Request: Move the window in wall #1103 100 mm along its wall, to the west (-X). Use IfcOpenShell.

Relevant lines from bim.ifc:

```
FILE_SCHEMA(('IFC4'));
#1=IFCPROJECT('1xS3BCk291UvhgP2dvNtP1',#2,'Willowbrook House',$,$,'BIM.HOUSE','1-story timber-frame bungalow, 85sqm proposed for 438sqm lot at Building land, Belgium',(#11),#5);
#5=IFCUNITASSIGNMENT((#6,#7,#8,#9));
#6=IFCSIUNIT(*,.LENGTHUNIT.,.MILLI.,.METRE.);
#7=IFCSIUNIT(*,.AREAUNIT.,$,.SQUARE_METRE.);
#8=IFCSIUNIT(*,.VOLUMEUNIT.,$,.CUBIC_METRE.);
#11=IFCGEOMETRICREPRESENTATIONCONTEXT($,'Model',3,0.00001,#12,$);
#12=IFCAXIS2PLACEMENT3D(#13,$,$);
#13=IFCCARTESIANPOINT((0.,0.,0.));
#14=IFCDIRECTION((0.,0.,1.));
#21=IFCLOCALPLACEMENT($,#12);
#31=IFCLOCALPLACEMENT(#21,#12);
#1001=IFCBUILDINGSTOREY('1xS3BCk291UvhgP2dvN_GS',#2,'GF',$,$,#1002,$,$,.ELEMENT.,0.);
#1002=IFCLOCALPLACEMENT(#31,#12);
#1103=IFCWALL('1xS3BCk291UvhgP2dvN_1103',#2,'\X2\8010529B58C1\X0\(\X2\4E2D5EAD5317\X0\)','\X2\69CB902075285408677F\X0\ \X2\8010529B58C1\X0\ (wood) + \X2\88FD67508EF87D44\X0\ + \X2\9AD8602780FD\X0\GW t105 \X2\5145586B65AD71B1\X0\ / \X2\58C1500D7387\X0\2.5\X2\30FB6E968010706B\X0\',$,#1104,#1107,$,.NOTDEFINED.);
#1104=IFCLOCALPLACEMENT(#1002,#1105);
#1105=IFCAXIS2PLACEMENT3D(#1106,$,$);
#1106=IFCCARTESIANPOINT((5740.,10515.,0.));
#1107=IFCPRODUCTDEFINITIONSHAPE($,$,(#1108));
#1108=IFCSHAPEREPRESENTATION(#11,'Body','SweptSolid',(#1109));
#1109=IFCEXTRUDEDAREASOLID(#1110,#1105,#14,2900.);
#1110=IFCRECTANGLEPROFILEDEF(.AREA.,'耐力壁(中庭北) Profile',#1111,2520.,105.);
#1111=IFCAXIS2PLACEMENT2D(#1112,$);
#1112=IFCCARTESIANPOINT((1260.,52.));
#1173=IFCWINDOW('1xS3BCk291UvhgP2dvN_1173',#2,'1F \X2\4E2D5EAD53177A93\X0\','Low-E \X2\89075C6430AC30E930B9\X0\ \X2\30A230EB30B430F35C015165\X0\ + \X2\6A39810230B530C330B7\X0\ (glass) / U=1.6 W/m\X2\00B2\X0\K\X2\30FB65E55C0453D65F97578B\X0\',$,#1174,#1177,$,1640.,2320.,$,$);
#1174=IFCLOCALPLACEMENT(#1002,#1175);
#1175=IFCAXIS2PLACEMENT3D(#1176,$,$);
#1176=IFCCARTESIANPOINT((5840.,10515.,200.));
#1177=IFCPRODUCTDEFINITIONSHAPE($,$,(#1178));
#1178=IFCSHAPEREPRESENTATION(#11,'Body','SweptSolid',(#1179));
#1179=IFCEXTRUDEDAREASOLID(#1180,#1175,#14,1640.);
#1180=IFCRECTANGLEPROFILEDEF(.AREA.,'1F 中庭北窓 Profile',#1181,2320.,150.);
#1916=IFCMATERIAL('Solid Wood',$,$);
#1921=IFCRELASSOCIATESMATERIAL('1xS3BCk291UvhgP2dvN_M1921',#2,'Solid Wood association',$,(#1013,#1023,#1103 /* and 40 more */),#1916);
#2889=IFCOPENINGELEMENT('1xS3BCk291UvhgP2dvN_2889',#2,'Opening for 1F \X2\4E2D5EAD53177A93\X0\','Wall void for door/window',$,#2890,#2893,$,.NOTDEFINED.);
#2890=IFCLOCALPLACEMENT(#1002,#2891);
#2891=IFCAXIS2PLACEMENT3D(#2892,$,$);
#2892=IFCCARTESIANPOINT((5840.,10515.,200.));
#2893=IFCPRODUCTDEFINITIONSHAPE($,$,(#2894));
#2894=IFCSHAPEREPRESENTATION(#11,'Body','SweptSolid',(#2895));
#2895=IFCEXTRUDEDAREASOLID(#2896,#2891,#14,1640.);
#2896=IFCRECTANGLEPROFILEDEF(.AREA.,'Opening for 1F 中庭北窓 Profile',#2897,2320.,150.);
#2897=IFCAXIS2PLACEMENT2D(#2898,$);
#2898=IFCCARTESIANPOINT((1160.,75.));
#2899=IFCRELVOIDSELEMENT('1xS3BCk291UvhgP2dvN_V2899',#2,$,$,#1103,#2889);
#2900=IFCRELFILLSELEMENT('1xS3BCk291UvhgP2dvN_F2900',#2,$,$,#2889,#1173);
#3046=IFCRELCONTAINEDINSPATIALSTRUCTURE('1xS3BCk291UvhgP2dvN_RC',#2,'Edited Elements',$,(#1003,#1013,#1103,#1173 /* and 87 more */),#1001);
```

```python
import ifcopenshell
import ifcopenshell.api.geometry
import ifcopenshell.util.placement

model = ifcopenshell.open("bim.ifc")

window = model.by_guid("1xS3BCk291UvhgP2dvN_1173")
opening = window.FillsVoids[0].RelatingOpeningElement
wall = opening.VoidsElements[0].RelatingBuildingElement

wall_matrix = ifcopenshell.util.placement.get_local_placement(wall.ObjectPlacement)
shift = wall_matrix[:3, 0] * -100.0
before = ifcopenshell.util.placement.get_local_placement(window.ObjectPlacement)[:3, 3].copy()

# The window is not placed relative to its opening, so move both.
for product in (opening, window):
    matrix = ifcopenshell.util.placement.get_local_placement(product.ObjectPlacement)
    matrix[:3, 3] += shift
    ifcopenshell.api.geometry.edit_object_placement(model, product=product, matrix=matrix, is_si=False)

after = ifcopenshell.util.placement.get_local_placement(window.ObjectPlacement)[:3, 3]
print("window moved by", (after - before).round(3) + 0.0)

model.write("bim_v2.ifc")
```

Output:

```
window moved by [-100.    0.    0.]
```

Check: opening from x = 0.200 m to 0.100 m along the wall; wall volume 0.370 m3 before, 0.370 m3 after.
